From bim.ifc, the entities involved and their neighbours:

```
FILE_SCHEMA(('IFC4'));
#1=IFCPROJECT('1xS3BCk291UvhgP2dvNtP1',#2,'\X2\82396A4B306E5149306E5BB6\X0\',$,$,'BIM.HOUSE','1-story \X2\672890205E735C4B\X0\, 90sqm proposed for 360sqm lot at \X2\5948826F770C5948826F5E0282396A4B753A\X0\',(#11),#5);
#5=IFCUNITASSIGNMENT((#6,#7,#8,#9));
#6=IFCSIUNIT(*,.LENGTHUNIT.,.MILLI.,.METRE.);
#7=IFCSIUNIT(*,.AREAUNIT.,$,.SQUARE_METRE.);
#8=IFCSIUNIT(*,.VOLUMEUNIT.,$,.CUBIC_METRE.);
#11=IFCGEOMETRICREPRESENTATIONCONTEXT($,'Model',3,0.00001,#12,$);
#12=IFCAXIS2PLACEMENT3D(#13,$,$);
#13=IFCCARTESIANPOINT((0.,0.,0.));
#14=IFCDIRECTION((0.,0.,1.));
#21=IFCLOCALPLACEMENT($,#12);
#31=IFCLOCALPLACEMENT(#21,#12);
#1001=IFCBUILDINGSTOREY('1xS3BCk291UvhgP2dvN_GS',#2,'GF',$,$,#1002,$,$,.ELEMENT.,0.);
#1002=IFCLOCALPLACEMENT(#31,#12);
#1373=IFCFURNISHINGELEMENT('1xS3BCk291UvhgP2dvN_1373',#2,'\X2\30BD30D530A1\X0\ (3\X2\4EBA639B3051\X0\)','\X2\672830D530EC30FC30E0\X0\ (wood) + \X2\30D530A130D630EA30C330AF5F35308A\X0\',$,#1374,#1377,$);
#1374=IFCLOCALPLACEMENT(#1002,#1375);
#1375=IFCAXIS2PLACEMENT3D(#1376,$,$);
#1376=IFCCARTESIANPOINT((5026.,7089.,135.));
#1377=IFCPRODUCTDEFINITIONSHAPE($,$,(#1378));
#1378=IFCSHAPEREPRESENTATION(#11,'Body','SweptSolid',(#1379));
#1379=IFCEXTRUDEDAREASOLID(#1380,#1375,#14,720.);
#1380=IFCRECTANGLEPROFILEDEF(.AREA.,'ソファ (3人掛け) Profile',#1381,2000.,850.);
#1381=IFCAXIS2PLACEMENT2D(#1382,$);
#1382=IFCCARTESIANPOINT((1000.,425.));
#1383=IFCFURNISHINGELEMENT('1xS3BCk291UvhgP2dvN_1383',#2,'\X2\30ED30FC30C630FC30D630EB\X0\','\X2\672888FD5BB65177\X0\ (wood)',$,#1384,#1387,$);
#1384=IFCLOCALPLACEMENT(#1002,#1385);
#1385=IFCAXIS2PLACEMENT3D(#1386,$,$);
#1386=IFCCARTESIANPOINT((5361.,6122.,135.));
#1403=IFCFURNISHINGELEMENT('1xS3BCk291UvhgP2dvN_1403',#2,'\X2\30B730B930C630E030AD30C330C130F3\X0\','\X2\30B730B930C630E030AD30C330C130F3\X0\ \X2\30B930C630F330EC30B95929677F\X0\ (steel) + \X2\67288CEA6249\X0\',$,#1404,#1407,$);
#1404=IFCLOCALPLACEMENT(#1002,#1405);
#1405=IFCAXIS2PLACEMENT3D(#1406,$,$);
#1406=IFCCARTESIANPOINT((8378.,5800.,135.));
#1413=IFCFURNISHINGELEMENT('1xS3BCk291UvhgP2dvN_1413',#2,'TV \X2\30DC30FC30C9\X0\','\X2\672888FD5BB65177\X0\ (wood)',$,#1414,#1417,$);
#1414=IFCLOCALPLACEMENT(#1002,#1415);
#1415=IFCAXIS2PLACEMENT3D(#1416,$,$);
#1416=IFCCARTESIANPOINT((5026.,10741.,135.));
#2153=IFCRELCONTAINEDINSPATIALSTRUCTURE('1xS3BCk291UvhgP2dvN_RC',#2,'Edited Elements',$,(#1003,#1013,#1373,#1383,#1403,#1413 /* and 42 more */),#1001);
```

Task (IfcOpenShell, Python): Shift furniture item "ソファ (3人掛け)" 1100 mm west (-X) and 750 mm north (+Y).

```python
import ifcopenshell
import ifcopenshell.api.geometry
import ifcopenshell.util.placement

model = ifcopenshell.open("bim.ifc")

item = model.by_guid("1xS3BCk291UvhgP2dvN_1373")
matrix = ifcopenshell.util.placement.get_local_placement(item.ObjectPlacement)
matrix[0, 3] -= 1100.0
matrix[1, 3] += 750.0
ifcopenshell.api.geometry.edit_object_placement(model, product=item, matrix=matrix, is_si=False)

print(ifcopenshell.util.placement.get_local_placement(item.ObjectPlacement).round(3) + 0.0)

model.write("bim_edited.ifc")
```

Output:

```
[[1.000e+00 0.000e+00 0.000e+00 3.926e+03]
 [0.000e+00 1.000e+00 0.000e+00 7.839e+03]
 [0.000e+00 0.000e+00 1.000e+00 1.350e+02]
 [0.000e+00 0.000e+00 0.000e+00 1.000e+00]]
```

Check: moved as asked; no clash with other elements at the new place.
